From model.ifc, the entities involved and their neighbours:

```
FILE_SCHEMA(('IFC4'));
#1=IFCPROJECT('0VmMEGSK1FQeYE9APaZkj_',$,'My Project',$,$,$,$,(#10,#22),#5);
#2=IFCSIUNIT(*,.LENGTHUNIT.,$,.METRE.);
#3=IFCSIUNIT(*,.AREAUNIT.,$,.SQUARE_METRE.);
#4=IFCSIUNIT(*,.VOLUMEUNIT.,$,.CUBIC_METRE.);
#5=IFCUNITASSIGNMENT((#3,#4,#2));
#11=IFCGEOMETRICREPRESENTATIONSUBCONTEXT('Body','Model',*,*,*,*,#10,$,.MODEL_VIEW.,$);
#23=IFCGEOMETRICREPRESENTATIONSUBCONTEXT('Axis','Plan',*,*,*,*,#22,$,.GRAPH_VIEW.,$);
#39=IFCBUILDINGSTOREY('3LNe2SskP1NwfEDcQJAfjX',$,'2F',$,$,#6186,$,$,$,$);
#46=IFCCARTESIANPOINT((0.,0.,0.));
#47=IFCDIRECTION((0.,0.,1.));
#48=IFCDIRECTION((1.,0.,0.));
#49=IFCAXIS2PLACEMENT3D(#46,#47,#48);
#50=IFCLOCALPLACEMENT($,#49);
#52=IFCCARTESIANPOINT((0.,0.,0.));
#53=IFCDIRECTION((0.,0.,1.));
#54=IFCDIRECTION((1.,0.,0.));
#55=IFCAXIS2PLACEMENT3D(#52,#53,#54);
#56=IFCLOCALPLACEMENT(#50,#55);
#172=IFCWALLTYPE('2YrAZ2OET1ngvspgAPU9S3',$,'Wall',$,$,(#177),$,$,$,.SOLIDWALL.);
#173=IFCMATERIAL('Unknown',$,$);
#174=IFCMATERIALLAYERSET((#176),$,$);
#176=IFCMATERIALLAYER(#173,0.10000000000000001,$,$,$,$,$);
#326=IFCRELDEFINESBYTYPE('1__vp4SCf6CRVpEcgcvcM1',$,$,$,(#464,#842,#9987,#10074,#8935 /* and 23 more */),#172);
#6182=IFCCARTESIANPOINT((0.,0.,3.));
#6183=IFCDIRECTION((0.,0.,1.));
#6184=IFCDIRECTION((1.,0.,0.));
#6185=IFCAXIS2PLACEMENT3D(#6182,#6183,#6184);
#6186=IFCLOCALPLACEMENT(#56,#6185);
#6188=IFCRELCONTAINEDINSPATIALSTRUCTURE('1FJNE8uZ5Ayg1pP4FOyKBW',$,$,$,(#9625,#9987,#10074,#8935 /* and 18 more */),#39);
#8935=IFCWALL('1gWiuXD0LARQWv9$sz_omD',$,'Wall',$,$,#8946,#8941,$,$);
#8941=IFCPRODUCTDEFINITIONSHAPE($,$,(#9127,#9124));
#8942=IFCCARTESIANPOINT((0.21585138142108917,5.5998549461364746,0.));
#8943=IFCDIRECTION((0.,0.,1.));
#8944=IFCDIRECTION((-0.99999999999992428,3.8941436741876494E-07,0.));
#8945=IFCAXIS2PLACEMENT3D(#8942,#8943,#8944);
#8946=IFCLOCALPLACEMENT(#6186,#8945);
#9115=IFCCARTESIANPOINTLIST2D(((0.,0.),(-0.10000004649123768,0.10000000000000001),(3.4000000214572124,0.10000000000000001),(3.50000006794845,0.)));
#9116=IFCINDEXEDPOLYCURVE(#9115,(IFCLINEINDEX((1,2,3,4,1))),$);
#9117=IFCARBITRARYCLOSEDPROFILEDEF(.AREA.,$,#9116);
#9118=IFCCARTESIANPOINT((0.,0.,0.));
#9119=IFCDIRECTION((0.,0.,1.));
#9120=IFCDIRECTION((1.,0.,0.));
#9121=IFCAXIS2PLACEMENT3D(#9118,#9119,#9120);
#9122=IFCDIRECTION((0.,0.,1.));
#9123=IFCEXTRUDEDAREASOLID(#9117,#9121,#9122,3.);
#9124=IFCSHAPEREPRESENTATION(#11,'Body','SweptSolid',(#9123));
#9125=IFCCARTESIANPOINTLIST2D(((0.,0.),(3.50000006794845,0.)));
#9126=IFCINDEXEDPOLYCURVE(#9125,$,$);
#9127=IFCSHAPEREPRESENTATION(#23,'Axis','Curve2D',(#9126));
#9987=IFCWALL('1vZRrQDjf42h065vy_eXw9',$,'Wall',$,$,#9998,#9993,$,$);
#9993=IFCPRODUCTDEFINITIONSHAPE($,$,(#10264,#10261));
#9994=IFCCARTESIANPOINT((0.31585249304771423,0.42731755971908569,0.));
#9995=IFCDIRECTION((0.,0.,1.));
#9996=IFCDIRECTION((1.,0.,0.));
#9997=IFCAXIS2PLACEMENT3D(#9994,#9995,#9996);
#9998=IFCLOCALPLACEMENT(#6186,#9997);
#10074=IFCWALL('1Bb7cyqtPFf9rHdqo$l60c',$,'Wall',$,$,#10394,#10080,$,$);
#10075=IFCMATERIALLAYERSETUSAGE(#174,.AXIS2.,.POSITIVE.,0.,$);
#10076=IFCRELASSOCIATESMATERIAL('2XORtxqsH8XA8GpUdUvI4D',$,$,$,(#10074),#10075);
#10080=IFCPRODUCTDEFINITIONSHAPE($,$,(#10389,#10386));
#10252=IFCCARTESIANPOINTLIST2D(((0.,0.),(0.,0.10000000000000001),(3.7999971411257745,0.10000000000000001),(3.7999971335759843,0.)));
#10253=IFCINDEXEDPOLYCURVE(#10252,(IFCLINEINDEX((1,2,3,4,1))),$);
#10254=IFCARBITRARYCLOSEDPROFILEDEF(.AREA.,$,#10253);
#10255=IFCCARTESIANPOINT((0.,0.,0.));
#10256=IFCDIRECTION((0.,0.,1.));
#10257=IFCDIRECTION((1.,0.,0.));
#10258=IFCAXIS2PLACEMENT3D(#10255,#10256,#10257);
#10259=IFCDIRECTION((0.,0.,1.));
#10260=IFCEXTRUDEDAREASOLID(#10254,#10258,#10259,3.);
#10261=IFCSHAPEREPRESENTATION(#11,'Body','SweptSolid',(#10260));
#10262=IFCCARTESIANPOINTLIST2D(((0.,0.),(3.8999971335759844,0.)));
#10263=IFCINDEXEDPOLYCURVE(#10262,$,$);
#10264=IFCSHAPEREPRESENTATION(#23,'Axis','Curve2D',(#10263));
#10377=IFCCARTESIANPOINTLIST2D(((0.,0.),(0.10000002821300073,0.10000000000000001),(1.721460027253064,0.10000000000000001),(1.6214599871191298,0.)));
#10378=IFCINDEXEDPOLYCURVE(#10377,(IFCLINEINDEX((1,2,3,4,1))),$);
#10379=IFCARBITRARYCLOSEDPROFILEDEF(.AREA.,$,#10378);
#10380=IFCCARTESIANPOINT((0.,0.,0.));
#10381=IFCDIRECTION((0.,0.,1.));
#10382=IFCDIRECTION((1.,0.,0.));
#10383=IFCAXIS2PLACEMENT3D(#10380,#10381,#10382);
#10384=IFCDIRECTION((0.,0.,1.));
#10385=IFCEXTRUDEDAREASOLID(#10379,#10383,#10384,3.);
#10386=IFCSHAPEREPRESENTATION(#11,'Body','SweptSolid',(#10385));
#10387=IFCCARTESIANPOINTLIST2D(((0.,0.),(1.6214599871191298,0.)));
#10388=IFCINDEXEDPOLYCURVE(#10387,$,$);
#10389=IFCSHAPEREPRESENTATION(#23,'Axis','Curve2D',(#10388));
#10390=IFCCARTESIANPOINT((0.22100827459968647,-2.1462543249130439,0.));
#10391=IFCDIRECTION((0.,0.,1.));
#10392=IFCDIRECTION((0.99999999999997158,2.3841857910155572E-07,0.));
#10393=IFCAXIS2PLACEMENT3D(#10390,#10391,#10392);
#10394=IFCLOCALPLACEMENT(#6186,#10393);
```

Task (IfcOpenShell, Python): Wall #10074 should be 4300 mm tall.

```python
import ifcopenshell
import ifcopenshell.geom
import ifcopenshell.util.representation
import ifcopenshell.util.shape

model = ifcopenshell.open("model.ifc")
settings = ifcopenshell.geom.settings()


def volume(element):
    """Net volume in cubic metres, openings subtracted."""
    shape = ifcopenshell.geom.create_shape(settings, element)
    return ifcopenshell.util.shape.get_volume(shape.geometry)


wall = model.by_guid("1Bb7cyqtPFf9rHdqo$l60c")
before = volume(wall)

body = ifcopenshell.util.representation.get_representation(wall, "Model", "Body")
solid = body.Items[0]
old_height = solid.Depth
solid.Depth = 4.3
after = volume(wall)

print(f"height {old_height:g} -> {solid.Depth:g}, volume {before:.3f} -> {after:.3f} m3")

model.write("model-out.ifc")
```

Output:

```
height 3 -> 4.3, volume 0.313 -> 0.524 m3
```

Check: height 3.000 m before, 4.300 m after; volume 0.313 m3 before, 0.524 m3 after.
